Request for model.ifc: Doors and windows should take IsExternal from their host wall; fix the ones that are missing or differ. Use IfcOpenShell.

First a look at what the model holds.

```python
import ifcopenshell
import ifcopenshell.util.element

model = ifcopenshell.open("model.ifc")
print(model.schema)
seen = {}
for e in model.by_type("IfcDoor") + model.by_type("IfcWindow"):
    if not e.FillsVoids:
        continue
    host = e.FillsVoids[0].RelatingOpeningElement.VoidsElements[0].RelatingBuildingElement
    own = ifcopenshell.util.element.get_pset(e, f"Pset_{e.is_a()[3:].removesuffix('StandardCase')}Common", "IsExternal")
    wall = ifcopenshell.util.element.get_pset(host, "Pset_WallCommon", "IsExternal")
    seen[e.is_a(), own, wall] = seen.get((e.is_a(), own, wall), 0) + 1
for (cls, own, wall), count in sorted(seen.items(), key=str):
    print(count, cls, "IsExternal:", own, "| host wall:", wall)
```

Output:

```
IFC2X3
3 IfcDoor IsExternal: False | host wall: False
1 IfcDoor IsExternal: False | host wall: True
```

```python
import ifcopenshell
import ifcopenshell.api.pset
import ifcopenshell.util.element

model = ifcopenshell.open("model.ifc")

count = 0
for ifc_class, pset_name in (("IfcDoor", "Pset_DoorCommon"), ("IfcWindow", "Pset_WindowCommon")):
    for e in model.by_type(ifc_class):
        if not e.FillsVoids:
            continue
        host = e.FillsVoids[0].RelatingOpeningElement.VoidsElements[0].RelatingBuildingElement
        external = ifcopenshell.util.element.get_pset(host, "Pset_WallCommon", "IsExternal")
        if external is None or ifcopenshell.util.element.get_pset(e, pset_name, "IsExternal") == external:
            continue
        pset = ifcopenshell.api.pset.add_pset(model, product=e, name=pset_name)
        ifcopenshell.api.pset.edit_pset(model, pset=pset, properties={"IsExternal": external})
        count += 1

print(count, "updated")

model.write("model_rev.ifc")
```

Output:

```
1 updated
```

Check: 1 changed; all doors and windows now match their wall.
